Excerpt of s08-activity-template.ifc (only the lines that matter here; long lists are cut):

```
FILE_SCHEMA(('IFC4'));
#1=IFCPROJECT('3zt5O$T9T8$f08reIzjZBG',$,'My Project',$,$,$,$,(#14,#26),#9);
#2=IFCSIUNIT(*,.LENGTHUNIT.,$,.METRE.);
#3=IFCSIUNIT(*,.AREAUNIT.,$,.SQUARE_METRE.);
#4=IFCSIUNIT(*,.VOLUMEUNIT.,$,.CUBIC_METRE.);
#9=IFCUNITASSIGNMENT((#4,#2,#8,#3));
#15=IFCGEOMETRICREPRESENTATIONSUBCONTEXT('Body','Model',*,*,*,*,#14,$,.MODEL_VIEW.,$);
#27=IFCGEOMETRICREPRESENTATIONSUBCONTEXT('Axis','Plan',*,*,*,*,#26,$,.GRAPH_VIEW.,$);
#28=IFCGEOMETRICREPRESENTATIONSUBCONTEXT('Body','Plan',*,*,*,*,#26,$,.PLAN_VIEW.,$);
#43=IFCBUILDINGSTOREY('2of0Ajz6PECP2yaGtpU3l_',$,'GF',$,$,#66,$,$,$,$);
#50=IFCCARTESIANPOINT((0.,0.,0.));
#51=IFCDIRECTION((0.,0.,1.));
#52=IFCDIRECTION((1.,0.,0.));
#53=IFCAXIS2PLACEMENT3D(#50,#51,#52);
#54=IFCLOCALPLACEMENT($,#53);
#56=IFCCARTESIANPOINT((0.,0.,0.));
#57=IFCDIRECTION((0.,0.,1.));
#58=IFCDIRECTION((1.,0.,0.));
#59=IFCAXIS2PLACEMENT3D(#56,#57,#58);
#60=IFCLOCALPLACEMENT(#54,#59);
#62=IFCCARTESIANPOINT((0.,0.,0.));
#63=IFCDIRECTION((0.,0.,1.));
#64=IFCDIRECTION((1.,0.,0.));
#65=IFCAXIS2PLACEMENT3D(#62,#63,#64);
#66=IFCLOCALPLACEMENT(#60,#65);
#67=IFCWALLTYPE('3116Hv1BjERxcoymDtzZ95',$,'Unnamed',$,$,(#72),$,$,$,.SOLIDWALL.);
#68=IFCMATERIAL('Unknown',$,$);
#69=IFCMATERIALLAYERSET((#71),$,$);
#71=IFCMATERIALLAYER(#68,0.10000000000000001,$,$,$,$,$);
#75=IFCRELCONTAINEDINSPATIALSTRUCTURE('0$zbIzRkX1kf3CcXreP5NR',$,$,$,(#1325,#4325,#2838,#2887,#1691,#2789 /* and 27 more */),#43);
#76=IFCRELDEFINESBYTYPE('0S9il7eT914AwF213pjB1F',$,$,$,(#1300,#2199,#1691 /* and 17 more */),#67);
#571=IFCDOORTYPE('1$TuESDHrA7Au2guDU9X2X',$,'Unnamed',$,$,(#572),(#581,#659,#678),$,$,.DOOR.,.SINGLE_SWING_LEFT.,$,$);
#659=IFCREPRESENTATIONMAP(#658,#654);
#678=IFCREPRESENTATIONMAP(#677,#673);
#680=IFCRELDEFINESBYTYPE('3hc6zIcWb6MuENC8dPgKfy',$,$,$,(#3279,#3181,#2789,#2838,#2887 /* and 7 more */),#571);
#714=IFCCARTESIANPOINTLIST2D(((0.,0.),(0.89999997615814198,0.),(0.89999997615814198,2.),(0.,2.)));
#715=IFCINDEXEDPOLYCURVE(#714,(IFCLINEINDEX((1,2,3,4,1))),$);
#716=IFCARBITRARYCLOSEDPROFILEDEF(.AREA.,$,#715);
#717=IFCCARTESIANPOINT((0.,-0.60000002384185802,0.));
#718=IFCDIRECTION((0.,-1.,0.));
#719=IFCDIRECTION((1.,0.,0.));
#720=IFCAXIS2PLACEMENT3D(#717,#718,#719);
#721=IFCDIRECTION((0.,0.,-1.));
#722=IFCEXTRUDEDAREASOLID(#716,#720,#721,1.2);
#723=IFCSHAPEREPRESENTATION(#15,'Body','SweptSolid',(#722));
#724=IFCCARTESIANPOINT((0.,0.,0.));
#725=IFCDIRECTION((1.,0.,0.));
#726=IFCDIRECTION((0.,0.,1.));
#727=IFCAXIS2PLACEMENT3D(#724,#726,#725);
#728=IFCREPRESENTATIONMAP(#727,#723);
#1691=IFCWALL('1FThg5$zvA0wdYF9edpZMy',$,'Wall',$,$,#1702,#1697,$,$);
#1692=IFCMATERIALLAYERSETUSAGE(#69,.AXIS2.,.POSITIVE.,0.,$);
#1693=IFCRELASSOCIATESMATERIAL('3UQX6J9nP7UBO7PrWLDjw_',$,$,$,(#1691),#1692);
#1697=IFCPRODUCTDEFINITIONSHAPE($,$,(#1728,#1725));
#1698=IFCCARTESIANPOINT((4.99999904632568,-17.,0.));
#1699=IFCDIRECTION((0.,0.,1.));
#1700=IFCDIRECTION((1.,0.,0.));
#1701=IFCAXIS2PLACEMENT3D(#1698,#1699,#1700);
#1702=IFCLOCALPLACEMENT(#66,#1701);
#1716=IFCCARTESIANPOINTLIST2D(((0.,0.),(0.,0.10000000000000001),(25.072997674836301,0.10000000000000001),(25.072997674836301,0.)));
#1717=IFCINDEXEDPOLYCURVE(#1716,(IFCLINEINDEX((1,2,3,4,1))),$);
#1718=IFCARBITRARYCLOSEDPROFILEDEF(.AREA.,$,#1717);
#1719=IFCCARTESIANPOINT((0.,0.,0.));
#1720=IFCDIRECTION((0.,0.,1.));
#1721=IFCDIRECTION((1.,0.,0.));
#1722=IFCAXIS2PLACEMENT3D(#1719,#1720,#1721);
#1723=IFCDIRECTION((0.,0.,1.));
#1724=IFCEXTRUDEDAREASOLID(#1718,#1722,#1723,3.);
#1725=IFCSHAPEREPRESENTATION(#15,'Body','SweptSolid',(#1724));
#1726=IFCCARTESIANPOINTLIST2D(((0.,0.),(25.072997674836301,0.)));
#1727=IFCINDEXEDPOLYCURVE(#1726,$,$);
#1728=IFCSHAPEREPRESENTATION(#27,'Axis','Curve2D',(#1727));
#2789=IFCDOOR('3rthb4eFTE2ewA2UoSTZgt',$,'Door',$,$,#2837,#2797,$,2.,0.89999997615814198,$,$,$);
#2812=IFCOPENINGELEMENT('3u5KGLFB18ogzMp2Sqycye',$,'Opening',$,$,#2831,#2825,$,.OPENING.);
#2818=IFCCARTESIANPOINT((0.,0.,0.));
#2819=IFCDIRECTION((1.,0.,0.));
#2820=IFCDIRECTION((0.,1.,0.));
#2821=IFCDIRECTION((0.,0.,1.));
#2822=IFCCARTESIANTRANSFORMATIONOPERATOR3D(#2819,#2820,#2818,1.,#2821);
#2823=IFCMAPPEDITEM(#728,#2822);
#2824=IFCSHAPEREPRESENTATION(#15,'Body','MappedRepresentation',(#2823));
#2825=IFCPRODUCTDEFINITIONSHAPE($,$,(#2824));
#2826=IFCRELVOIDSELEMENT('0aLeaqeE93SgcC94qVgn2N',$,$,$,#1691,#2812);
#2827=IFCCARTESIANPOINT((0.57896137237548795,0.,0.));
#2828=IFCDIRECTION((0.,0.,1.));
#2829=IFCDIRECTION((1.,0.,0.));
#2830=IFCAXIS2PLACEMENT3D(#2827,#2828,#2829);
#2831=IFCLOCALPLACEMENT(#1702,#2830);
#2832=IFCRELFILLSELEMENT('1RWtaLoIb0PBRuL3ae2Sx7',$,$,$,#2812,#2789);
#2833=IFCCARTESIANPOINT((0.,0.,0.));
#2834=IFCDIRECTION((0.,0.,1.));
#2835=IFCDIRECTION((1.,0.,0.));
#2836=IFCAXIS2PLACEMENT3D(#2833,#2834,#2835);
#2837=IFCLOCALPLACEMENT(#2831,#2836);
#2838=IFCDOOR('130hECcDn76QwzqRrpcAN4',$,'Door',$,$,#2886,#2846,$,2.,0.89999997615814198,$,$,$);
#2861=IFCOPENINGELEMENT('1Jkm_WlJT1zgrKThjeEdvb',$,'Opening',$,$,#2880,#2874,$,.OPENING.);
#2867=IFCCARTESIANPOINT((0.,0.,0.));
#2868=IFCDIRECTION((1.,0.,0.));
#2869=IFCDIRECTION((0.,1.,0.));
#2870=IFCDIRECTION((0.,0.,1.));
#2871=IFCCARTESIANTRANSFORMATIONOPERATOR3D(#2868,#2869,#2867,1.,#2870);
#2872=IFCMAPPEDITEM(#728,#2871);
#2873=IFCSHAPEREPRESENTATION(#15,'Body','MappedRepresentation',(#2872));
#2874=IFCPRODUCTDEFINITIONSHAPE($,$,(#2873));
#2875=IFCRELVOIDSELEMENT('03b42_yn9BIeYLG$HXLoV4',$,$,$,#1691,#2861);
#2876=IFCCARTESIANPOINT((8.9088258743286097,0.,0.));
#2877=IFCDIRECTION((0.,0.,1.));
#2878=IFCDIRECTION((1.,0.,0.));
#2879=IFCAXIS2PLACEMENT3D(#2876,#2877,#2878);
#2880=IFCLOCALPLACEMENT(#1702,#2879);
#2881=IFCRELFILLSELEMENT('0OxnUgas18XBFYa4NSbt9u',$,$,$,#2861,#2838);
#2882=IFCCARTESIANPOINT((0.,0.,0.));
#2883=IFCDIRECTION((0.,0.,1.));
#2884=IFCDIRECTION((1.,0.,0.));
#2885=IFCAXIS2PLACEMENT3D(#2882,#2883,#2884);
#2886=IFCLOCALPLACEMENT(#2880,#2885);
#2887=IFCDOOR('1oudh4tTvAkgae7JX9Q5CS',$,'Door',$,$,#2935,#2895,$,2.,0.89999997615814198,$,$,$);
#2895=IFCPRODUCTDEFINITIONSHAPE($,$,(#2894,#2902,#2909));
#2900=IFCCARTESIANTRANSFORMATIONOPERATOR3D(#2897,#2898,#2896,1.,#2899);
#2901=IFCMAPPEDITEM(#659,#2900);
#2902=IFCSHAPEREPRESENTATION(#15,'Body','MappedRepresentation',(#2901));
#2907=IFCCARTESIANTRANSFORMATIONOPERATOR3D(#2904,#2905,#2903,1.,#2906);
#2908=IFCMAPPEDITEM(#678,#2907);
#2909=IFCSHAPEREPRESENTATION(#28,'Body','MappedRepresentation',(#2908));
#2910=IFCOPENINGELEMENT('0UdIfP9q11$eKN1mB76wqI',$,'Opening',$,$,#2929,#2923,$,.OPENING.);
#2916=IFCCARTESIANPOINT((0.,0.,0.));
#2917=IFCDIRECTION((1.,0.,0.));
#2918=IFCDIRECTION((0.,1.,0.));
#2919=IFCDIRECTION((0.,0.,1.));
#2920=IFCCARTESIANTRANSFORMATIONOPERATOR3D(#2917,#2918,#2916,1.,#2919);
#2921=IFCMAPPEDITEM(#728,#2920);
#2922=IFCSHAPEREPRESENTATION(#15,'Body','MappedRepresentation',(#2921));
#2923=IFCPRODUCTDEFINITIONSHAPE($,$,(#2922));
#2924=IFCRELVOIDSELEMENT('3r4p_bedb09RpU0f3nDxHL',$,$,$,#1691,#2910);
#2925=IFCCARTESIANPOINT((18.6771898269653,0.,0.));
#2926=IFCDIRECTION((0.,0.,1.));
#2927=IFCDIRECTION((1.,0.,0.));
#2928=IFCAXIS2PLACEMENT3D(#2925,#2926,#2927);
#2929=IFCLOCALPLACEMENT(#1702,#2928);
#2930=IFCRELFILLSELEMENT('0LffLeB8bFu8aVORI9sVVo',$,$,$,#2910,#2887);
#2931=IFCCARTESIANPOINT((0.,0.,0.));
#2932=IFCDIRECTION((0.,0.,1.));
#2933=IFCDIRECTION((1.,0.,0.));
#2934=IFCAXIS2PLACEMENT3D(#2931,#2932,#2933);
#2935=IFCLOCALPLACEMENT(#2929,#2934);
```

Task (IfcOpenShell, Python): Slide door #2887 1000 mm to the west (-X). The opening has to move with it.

```python
import ifcopenshell
import ifcopenshell.api.geometry
import ifcopenshell.util.placement
import ifcopenshell.util.unit

model = ifcopenshell.open("s08-activity-template.ifc")
unit_scale = ifcopenshell.util.unit.calculate_unit_scale(model)

door = model.by_guid("1oudh4tTvAkgae7JX9Q5CS")
opening = door.FillsVoids[0].RelatingOpeningElement
wall = opening.VoidsElements[0].RelatingBuildingElement

wall_matrix = ifcopenshell.util.placement.get_local_placement(wall.ObjectPlacement)
shift = wall_matrix[:3, 0] * -1 / unit_scale
before = ifcopenshell.util.placement.get_local_placement(door.ObjectPlacement)[:3, 3].copy()

# The door is placed relative to its opening, so it follows when the opening moves.
matrix = ifcopenshell.util.placement.get_local_placement(opening.ObjectPlacement)
matrix[:3, 3] += shift
ifcopenshell.api.geometry.edit_object_placement(
    model, product=opening, matrix=matrix, is_si=False, should_transform_children=True
)

after = ifcopenshell.util.placement.get_local_placement(door.ObjectPlacement)[:3, 3]
print("door moved by", (after - before).round(3) + 0.0)

model.write("s08-activity-template_edited.ifc")
```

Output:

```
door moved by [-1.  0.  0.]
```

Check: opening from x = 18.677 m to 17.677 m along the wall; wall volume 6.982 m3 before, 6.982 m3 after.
